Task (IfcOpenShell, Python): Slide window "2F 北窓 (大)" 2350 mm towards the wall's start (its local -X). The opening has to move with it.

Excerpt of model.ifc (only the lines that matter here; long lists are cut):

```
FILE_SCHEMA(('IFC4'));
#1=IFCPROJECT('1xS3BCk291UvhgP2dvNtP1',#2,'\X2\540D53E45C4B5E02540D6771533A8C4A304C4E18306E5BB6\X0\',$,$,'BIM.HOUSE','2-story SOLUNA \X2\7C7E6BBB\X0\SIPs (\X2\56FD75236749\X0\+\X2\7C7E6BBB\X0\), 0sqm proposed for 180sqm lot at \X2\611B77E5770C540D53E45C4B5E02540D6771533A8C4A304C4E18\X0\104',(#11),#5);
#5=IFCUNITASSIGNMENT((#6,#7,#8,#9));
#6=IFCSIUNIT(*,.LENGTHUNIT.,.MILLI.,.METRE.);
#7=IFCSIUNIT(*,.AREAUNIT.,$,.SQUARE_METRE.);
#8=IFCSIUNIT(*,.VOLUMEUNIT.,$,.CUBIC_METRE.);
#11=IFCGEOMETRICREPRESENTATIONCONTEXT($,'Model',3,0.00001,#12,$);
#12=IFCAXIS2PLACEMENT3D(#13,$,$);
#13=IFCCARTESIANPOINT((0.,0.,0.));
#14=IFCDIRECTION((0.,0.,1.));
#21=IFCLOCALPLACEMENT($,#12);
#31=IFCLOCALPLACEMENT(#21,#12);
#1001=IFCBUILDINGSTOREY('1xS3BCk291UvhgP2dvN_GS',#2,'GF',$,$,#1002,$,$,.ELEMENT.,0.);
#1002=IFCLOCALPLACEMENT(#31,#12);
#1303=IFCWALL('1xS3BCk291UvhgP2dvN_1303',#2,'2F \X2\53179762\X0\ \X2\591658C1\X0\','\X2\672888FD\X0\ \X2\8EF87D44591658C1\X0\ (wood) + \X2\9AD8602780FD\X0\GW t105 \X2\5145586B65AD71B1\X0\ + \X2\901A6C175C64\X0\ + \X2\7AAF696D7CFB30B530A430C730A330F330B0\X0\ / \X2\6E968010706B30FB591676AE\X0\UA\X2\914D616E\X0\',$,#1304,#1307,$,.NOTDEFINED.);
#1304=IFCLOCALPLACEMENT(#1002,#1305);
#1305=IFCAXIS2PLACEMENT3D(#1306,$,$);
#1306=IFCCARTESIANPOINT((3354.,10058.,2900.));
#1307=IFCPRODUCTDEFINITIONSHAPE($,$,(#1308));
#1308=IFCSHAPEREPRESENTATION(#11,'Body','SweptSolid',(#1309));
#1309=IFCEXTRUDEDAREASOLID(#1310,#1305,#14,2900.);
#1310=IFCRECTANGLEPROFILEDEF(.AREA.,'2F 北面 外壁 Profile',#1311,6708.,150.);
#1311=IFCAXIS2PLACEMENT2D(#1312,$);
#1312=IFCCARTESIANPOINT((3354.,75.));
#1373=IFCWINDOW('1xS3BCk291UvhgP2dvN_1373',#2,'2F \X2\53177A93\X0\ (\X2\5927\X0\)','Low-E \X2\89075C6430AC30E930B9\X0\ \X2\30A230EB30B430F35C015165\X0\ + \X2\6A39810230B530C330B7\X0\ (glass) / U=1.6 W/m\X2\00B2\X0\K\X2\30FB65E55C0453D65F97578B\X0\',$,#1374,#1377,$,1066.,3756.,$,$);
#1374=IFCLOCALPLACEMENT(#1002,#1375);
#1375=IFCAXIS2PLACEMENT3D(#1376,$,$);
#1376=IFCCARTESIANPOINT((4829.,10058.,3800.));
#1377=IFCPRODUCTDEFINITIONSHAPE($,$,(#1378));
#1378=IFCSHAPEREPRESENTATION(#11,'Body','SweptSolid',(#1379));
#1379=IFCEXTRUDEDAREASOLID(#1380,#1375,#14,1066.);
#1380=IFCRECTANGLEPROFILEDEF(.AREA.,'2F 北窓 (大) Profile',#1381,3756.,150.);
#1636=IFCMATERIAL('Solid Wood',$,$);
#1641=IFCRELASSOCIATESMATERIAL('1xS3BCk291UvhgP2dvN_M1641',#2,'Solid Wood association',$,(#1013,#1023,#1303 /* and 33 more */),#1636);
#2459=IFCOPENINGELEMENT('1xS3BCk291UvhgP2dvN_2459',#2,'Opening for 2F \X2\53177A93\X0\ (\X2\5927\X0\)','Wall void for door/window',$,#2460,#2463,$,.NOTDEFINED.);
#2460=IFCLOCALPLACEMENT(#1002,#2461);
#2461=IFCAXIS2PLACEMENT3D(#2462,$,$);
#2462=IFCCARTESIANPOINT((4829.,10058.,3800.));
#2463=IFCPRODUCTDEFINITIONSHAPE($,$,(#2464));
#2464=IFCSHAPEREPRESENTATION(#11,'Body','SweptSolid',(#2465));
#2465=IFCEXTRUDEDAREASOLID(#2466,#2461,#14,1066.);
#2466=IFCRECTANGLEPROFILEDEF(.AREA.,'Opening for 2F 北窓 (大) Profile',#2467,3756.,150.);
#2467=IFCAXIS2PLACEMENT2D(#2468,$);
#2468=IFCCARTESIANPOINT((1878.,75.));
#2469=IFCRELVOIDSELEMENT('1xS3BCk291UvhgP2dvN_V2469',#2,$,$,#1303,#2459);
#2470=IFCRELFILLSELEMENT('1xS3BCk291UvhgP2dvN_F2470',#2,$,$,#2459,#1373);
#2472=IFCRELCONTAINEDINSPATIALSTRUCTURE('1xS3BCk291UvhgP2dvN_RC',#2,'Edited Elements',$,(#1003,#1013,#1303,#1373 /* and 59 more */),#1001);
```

```python
import ifcopenshell
import ifcopenshell.api.geometry
import ifcopenshell.util.placement
import ifcopenshell.util.unit

model = ifcopenshell.open("model.ifc")
unit_scale = ifcopenshell.util.unit.calculate_unit_scale(model)

window = model.by_guid("1xS3BCk291UvhgP2dvN_1373")
opening = window.FillsVoids[0].RelatingOpeningElement
wall = opening.VoidsElements[0].RelatingBuildingElement

wall_matrix = ifcopenshell.util.placement.get_local_placement(wall.ObjectPlacement)
shift = wall_matrix[:3, 0] * -2.35 / unit_scale
before = ifcopenshell.util.placement.get_local_placement(window.ObjectPlacement)[:3, 3].copy()

# The window is not placed relative to its opening, so move both.
for product in (opening, window):
    matrix = ifcopenshell.util.placement.get_local_placement(product.ObjectPlacement)
    matrix[:3, 3] += shift
    ifcopenshell.api.geometry.edit_object_placement(model, product=product, matrix=matrix, is_si=False)

after = ifcopenshell.util.placement.get_local_placement(window.ObjectPlacement)[:3, 3]
print("window moved by", (after - before).round(3) + 0.0)

model.write("model_updated.ifc")
```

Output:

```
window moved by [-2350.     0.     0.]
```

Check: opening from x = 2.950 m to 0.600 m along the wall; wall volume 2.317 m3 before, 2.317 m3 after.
